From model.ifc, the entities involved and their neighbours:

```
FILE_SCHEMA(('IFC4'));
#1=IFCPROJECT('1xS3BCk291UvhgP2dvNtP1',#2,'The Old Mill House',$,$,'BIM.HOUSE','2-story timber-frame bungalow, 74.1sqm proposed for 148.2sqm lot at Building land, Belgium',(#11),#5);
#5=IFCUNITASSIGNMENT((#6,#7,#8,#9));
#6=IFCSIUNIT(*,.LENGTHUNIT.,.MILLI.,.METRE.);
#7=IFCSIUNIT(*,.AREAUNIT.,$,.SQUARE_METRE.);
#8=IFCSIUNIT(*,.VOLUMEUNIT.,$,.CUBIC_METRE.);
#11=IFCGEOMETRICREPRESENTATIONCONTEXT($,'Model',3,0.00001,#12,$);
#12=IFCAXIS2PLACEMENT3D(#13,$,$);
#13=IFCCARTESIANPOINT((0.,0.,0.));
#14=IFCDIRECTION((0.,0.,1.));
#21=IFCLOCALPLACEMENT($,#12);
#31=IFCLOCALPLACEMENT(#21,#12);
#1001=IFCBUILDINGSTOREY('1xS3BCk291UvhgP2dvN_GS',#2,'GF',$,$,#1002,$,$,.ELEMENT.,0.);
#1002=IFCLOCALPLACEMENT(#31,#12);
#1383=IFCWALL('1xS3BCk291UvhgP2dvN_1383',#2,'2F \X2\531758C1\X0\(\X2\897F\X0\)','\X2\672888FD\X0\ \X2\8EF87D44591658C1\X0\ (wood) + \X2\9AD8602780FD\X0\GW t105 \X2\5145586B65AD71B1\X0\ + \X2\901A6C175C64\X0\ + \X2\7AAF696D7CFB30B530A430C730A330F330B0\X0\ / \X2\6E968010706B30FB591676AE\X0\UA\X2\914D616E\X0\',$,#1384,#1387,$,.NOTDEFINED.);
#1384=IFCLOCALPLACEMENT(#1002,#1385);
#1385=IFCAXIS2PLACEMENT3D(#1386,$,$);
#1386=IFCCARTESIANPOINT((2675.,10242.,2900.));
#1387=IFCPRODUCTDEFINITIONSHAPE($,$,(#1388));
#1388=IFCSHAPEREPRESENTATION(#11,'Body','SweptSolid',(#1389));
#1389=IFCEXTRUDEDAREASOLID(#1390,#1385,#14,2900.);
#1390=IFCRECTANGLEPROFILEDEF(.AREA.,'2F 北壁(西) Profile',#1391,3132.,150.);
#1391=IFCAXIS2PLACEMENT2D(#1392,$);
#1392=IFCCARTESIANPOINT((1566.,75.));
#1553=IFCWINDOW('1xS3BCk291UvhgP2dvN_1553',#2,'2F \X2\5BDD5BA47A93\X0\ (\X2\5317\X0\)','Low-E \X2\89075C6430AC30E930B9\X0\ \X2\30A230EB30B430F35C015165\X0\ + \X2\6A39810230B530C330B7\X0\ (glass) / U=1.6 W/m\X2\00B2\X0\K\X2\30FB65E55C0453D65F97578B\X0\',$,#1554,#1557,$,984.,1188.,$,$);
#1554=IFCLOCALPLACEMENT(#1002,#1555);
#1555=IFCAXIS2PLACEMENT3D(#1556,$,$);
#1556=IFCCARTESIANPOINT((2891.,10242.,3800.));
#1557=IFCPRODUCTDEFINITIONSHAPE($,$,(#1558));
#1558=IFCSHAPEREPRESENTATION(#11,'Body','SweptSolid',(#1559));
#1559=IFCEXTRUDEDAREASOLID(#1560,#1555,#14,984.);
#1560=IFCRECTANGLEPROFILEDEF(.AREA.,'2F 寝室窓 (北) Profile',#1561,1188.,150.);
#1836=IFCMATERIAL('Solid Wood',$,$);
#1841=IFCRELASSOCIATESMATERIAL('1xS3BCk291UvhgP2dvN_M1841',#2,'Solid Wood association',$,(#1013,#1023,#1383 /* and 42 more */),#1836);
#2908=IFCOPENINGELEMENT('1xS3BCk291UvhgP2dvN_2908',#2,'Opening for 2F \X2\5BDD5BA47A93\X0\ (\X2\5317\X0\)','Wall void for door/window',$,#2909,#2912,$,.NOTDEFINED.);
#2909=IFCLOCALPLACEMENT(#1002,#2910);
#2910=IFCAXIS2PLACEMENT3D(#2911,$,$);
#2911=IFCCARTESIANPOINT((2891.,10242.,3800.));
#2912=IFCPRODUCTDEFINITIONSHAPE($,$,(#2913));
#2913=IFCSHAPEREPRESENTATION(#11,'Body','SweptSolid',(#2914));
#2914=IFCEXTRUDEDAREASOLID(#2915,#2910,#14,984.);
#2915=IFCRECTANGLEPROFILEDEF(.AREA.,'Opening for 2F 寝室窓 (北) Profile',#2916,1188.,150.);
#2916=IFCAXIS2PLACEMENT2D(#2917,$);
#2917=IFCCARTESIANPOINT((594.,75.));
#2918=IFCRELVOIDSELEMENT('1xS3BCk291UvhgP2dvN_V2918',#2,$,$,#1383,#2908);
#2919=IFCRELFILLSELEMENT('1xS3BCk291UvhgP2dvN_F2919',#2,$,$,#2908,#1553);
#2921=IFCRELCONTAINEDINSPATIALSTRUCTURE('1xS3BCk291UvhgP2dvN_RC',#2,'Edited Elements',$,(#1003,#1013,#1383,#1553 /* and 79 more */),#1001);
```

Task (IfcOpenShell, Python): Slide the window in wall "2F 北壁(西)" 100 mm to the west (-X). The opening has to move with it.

```python
import ifcopenshell
import ifcopenshell.api.geometry
import ifcopenshell.util.placement
import ifcopenshell.util.unit

model = ifcopenshell.open("model.ifc")
unit_scale = ifcopenshell.util.unit.calculate_unit_scale(model)

window = model.by_id(1553)
opening = window.FillsVoids[0].RelatingOpeningElement
wall = opening.VoidsElements[0].RelatingBuildingElement

wall_matrix = ifcopenshell.util.placement.get_local_placement(wall.ObjectPlacement)
shift = wall_matrix[:3, 0] * -0.1 / unit_scale
before = ifcopenshell.util.placement.get_local_placement(window.ObjectPlacement)[:3, 3].copy()

# The window is not placed relative to its opening, so move both.
for product in (opening, window):
    matrix = ifcopenshell.util.placement.get_local_placement(product.ObjectPlacement)
    matrix[:3, 3] += shift
    ifcopenshell.api.geometry.edit_object_placement(model, product=product, matrix=matrix, is_si=False)

after = ifcopenshell.util.placement.get_local_placement(window.ObjectPlacement)[:3, 3]
print("window moved by", (after - before).round(3) + 0.0)

model.write("model_edited.ifc")
```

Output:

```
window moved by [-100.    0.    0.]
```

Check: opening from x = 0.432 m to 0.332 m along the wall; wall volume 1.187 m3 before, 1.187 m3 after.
